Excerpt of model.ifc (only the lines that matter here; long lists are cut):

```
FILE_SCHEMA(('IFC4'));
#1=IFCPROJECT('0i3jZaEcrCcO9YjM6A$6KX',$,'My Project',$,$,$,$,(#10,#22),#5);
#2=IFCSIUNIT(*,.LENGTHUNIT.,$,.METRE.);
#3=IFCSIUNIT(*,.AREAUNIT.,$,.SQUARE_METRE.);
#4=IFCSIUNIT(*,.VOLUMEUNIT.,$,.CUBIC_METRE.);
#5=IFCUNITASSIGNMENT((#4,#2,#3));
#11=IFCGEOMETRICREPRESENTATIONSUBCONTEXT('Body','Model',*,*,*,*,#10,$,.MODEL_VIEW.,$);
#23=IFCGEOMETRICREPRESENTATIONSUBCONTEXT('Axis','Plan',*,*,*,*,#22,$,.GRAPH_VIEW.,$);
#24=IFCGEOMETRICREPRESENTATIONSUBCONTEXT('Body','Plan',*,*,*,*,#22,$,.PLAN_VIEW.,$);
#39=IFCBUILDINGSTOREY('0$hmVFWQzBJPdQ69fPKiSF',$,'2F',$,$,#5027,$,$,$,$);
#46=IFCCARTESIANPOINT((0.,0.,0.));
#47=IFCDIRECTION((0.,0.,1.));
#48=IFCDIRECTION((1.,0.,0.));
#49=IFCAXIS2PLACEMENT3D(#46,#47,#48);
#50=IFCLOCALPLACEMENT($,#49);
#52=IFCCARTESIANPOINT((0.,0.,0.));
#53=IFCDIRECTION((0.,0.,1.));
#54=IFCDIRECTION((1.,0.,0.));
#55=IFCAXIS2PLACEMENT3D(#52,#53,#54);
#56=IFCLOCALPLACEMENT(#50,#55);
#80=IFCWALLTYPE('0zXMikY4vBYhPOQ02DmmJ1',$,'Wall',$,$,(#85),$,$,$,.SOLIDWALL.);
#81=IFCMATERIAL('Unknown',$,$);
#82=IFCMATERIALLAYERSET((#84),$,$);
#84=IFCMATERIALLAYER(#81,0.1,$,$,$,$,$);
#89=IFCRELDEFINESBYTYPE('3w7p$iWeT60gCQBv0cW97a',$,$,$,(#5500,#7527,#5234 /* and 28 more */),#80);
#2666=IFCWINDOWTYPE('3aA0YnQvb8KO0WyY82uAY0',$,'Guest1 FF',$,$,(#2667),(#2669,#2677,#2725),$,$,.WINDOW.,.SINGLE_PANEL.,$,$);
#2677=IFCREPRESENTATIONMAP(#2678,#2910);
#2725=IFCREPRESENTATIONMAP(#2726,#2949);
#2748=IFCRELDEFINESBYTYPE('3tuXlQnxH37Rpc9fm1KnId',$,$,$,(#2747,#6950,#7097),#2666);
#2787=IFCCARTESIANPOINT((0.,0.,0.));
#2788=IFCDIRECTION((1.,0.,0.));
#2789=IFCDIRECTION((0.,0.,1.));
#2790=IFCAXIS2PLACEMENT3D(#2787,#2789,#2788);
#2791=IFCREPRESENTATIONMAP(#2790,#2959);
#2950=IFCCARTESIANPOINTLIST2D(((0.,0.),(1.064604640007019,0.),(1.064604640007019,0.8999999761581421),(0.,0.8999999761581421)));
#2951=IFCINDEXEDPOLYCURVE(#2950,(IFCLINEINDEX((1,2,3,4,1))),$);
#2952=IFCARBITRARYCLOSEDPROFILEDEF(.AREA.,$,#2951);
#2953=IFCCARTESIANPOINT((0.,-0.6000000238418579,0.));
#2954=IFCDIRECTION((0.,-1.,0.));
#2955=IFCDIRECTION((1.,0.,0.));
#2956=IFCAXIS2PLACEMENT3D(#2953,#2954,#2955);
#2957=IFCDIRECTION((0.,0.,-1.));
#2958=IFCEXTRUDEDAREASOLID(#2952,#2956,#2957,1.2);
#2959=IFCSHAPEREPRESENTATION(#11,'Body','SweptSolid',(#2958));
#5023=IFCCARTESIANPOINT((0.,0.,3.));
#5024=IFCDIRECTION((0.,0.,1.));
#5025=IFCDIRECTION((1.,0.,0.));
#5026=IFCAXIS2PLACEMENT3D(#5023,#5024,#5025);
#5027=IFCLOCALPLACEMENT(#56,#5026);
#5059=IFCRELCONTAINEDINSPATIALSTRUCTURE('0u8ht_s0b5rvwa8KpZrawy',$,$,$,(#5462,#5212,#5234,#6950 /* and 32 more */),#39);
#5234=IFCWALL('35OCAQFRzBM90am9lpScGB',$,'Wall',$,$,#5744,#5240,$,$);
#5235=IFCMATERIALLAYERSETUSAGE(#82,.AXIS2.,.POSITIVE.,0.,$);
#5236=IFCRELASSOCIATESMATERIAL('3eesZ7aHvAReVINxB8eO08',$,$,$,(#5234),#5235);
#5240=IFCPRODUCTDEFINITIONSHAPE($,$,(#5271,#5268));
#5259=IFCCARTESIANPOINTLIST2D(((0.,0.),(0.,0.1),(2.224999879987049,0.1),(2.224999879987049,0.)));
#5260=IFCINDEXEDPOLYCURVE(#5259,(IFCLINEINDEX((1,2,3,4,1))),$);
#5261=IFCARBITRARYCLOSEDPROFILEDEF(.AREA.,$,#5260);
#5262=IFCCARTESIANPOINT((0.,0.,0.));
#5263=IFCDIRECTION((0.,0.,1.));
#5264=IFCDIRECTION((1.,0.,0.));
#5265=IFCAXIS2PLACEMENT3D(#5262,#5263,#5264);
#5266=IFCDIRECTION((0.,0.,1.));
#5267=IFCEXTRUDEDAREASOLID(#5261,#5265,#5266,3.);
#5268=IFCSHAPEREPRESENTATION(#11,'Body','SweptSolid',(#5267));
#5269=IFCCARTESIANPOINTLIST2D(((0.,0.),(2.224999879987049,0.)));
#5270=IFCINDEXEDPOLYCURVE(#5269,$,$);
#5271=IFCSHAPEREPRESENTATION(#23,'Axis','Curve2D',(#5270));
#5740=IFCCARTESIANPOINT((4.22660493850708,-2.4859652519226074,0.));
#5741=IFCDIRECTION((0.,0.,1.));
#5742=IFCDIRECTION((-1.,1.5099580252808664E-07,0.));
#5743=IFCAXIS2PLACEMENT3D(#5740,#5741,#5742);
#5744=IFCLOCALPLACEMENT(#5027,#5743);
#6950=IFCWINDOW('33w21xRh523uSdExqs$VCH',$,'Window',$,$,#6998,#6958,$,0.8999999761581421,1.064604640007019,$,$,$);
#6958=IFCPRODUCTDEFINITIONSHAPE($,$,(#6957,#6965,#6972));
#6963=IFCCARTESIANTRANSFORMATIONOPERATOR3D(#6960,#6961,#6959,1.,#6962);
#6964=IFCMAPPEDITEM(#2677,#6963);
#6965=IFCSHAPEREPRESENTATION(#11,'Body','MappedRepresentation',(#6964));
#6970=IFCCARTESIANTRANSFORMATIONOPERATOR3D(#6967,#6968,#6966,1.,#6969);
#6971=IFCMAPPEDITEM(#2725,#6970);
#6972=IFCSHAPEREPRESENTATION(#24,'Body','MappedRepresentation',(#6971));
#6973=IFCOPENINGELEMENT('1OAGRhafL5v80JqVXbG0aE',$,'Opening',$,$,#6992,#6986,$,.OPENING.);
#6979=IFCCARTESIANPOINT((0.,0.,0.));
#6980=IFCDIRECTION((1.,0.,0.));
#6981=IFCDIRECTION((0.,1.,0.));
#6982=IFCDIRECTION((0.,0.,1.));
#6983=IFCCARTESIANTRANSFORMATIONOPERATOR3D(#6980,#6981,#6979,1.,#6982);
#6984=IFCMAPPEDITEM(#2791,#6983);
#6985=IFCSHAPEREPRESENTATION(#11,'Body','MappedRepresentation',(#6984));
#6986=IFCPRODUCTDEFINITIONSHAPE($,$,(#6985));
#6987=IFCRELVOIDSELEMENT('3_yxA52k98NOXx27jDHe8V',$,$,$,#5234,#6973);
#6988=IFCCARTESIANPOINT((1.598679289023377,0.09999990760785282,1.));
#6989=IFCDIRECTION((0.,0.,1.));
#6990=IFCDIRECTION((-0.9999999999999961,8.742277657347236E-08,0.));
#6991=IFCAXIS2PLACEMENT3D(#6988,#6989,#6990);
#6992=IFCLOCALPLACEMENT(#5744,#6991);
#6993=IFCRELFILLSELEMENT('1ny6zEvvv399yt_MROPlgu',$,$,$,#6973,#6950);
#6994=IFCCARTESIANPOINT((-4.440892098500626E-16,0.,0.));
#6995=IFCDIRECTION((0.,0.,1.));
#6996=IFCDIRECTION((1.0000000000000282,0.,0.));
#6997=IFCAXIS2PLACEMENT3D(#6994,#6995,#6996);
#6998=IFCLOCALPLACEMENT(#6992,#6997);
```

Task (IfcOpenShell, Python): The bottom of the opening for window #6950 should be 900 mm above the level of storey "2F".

```python
import numpy as np
import ifcopenshell
import ifcopenshell.api.geometry
import ifcopenshell.geom
import ifcopenshell.util.element
import ifcopenshell.util.placement
import ifcopenshell.util.shape
import ifcopenshell.util.unit

model = ifcopenshell.open("model.ifc")
unit_scale = ifcopenshell.util.unit.calculate_unit_scale(model)

window = model.by_guid("33w21xRh523uSdExqs$VCH")
opening = window.FillsVoids[0].RelatingOpeningElement
storey = ifcopenshell.util.element.get_container(window, ifc_class="IfcBuildingStorey")
level = ifcopenshell.util.placement.get_local_placement(storey.ObjectPlacement)[2, 3]

# The opening's origin need not be at the sill, so measure its lowest point.
shape = ifcopenshell.geom.create_shape(ifcopenshell.geom.settings(), opening)
bottom = ifcopenshell.util.shape.get_shape_bottom_elevation(shape, shape.geometry) / unit_scale
dz = level + 0.9 / unit_scale - bottom

shift = np.array([0.0, 0.0, dz])
# The window is placed relative to its opening, so it follows when the opening moves.
matrix = ifcopenshell.util.placement.get_local_placement(opening.ObjectPlacement)
matrix[:3, 3] += shift
ifcopenshell.api.geometry.edit_object_placement(
    model, product=opening, matrix=matrix, is_si=False, should_transform_children=True
)

print(f"moved by {dz * unit_scale:+.3f} m")

model.write("model_updated.ifc")
```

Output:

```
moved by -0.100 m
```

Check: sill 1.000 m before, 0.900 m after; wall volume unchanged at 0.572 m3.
